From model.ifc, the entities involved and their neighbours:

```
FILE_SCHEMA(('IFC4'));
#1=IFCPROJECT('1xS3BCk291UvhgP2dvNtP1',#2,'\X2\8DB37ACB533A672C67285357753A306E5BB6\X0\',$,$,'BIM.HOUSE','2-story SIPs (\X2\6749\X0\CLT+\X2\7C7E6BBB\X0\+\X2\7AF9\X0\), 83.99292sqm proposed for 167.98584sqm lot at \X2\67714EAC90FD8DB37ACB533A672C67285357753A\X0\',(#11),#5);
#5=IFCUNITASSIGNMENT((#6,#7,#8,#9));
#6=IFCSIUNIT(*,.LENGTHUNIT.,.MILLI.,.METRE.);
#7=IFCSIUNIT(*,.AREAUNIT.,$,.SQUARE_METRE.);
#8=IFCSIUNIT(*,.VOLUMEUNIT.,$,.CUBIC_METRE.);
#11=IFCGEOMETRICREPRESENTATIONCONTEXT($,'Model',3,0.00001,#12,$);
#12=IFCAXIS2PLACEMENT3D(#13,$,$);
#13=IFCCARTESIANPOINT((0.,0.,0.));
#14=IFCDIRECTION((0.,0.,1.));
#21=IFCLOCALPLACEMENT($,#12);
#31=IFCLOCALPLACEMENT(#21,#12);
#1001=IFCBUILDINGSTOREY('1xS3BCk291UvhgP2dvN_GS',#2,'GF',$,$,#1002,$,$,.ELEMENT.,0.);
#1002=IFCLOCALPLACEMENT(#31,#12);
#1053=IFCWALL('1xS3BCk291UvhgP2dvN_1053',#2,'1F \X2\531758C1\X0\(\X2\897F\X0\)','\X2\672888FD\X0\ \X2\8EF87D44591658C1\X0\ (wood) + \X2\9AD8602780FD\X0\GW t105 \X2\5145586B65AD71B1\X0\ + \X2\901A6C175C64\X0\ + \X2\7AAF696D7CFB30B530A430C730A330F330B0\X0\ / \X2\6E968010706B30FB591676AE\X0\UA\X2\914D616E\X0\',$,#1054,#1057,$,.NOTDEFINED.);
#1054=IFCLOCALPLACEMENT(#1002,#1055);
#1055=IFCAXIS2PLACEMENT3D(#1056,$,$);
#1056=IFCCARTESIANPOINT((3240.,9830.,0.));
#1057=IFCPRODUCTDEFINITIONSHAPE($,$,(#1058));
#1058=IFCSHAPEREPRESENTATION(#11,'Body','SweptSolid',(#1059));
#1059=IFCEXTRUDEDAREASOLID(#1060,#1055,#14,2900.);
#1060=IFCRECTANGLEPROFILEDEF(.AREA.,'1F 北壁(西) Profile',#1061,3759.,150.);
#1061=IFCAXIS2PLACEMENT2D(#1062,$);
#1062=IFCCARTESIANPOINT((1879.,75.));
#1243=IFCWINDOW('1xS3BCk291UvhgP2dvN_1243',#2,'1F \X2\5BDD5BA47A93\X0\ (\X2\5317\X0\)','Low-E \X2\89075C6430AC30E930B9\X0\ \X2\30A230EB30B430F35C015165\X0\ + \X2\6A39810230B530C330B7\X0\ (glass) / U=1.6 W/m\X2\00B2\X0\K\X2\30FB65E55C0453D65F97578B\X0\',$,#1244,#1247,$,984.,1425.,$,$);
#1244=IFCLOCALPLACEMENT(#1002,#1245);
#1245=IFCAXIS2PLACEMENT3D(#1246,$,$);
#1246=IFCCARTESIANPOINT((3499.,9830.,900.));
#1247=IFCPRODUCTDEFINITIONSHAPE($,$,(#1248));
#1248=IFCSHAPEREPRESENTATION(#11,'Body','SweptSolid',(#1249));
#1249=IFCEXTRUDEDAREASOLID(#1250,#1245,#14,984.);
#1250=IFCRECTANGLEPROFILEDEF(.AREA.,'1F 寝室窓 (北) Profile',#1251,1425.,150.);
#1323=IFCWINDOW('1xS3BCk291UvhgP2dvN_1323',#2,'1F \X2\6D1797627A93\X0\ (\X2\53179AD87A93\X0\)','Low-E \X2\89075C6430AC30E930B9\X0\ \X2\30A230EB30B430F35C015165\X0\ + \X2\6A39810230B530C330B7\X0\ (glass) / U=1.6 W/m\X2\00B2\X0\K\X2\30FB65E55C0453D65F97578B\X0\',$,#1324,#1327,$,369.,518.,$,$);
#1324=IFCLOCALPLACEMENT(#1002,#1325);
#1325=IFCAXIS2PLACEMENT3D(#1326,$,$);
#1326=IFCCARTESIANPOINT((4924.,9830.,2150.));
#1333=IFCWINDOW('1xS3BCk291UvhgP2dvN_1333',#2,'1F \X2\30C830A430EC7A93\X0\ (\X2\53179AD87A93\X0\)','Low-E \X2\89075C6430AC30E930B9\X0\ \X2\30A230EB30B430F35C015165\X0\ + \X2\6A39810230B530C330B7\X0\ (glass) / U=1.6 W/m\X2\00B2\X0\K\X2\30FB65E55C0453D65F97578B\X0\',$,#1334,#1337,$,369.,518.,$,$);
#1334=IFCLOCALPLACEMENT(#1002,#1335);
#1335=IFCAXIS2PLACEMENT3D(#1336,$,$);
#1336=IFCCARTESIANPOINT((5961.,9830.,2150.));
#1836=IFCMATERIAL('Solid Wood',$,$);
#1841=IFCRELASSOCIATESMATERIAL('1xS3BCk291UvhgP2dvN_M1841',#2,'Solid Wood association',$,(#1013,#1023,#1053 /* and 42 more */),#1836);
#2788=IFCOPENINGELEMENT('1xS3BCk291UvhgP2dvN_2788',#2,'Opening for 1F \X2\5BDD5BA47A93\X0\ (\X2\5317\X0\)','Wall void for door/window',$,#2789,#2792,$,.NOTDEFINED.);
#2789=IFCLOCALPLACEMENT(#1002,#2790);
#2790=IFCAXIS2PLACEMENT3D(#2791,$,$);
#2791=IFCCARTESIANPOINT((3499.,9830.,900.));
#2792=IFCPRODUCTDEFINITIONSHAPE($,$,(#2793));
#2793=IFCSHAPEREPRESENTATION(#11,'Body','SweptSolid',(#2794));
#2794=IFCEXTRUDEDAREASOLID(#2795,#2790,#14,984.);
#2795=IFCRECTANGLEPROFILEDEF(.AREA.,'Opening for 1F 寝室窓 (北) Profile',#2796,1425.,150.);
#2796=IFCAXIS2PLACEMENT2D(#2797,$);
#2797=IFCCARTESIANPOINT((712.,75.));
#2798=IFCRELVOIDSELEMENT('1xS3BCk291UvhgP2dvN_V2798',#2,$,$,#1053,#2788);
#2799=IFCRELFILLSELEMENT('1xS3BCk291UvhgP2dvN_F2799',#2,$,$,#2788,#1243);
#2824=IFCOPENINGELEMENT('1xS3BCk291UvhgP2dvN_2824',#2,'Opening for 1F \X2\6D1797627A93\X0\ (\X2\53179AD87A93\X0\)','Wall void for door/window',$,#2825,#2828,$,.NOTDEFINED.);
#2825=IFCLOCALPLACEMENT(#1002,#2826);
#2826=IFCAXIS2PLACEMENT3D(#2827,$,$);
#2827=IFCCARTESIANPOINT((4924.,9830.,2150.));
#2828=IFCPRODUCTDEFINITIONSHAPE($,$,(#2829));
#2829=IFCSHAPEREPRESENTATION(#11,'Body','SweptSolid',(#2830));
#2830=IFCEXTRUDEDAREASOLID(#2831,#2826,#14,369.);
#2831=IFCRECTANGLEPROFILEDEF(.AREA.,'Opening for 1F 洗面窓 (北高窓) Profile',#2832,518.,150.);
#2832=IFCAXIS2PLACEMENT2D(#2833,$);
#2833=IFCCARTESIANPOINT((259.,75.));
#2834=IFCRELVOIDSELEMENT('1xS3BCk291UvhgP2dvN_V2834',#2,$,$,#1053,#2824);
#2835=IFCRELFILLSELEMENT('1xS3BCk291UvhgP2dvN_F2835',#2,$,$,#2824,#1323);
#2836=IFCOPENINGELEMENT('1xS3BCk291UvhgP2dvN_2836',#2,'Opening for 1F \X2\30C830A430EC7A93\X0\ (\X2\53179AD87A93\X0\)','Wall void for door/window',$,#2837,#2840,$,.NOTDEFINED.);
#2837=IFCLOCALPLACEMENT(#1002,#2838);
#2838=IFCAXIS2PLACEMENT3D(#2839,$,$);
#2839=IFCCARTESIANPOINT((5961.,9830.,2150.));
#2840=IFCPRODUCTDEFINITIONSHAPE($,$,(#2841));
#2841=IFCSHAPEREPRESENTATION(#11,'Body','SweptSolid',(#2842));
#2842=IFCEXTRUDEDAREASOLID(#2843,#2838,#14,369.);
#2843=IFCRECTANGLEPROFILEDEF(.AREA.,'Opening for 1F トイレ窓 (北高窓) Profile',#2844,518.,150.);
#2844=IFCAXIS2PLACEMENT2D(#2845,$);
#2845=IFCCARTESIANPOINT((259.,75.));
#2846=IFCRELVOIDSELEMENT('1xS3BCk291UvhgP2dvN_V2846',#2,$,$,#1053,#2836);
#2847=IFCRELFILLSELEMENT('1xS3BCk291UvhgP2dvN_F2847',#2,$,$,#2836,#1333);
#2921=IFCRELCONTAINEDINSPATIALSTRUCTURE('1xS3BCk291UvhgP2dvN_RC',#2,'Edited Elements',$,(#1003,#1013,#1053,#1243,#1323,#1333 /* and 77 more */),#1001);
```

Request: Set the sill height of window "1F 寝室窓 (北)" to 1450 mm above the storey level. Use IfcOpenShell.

```python
import numpy as np
import ifcopenshell
import ifcopenshell.api.geometry
import ifcopenshell.geom
import ifcopenshell.util.element
import ifcopenshell.util.placement
import ifcopenshell.util.shape
import ifcopenshell.util.unit

model = ifcopenshell.open("model.ifc")
unit_scale = ifcopenshell.util.unit.calculate_unit_scale(model)

window = model.by_id(1243)
opening = window.FillsVoids[0].RelatingOpeningElement
storey = ifcopenshell.util.element.get_container(window, ifc_class="IfcBuildingStorey")
level = ifcopenshell.util.placement.get_local_placement(storey.ObjectPlacement)[2, 3]

# The opening's origin need not be at the sill, so measure its lowest point.
shape = ifcopenshell.geom.create_shape(ifcopenshell.geom.settings(), opening)
bottom = ifcopenshell.util.shape.get_shape_bottom_elevation(shape, shape.geometry) / unit_scale
dz = level + 1450.0 - bottom

shift = np.array([0.0, 0.0, dz])
# The window is not placed relative to its opening, so move both.
for product in (opening, window):
    matrix = ifcopenshell.util.placement.get_local_placement(product.ObjectPlacement)
    matrix[:3, 3] += shift
    ifcopenshell.api.geometry.edit_object_placement(model, product=product, matrix=matrix, is_si=False)

print(f"moved by {dz * unit_scale:+.3f} m")

model.write("model_edited.ifc")
```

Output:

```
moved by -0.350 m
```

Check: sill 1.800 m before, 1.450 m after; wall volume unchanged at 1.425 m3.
